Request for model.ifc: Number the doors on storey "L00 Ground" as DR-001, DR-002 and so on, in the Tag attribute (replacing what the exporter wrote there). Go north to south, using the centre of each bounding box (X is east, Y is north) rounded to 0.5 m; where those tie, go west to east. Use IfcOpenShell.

First a look at what the model holds.

```python
import ifcopenshell
import ifcopenshell.util.element
import ifcopenshell.util.placement

model = ifcopenshell.open("model.ifc")
print(model.schema)
storey = next(s for s in model.by_type("IfcBuildingStorey") if s.Name == "L00 Ground")
doors = [e for e in ifcopenshell.util.element.get_decomposition(storey) if e.is_a("IfcDoor")]
for e in sorted(doors, key=lambda e: e.id()):
    origin = ifcopenshell.util.placement.get_local_placement(e.ObjectPlacement)[:3, 3]
    print(e.id(), e.Tag, e.Name, origin.round(2) + 0.0, sep=" | ")
```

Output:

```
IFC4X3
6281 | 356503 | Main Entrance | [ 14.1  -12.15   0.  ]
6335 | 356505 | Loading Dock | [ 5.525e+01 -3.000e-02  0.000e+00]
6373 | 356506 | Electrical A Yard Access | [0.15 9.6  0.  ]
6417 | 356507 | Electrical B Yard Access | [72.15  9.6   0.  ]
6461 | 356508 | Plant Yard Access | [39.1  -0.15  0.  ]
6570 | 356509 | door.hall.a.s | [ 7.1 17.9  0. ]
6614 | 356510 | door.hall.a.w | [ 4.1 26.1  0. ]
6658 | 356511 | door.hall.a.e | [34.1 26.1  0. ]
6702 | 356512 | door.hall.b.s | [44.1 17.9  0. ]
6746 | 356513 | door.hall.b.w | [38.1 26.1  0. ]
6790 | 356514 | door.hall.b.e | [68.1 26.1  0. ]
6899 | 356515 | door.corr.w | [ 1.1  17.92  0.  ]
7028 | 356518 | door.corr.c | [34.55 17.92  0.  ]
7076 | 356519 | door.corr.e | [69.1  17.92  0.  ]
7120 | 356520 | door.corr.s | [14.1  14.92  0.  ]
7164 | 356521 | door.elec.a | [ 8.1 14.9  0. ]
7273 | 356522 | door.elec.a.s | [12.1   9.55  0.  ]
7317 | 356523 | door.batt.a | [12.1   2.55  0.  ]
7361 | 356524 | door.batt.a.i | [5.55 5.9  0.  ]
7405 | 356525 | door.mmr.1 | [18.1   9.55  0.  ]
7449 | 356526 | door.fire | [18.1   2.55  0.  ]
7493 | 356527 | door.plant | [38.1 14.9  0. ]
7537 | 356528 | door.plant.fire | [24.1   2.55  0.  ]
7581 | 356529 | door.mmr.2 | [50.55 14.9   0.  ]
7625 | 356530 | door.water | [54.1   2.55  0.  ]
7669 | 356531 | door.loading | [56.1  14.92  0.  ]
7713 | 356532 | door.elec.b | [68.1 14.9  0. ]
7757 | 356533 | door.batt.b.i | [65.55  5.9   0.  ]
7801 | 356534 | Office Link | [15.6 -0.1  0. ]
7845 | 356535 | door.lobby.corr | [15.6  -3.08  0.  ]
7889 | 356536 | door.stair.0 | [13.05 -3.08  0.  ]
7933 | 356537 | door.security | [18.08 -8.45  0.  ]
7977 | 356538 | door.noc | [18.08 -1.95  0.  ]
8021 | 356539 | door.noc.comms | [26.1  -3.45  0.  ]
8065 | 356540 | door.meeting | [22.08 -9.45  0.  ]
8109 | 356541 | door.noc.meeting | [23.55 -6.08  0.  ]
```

```python
import ifcopenshell
import ifcopenshell.geom
import ifcopenshell.util.element
import ifcopenshell.util.shape

model = ifcopenshell.open("model.ifc")
settings = ifcopenshell.geom.settings()
settings.set("use-world-coords", True)


def centre(element):
    shape = ifcopenshell.geom.create_shape(settings, element)
    return ifcopenshell.util.shape.get_bbox_centroid(shape.geometry)


storey = next(s for s in model.by_type("IfcBuildingStorey") if s.Name == "L00 Ground")
doors = [e for e in ifcopenshell.util.element.get_decomposition(storey) if e.is_a("IfcDoor")]

# Insertion points can sit at a corner or the storey origin, so sort by the geometry (in metres).
centres = {e: centre(e) for e in doors}
doors.sort(key=lambda e: (-round(centres[e][1] / 0.5), centres[e][0]))

for i, e in enumerate(doors, start=1):
    number = f"DR-0{i:02d}"
    e.Tag = number
    print(e.id(), number)

model.write("model_updated.ifc")
```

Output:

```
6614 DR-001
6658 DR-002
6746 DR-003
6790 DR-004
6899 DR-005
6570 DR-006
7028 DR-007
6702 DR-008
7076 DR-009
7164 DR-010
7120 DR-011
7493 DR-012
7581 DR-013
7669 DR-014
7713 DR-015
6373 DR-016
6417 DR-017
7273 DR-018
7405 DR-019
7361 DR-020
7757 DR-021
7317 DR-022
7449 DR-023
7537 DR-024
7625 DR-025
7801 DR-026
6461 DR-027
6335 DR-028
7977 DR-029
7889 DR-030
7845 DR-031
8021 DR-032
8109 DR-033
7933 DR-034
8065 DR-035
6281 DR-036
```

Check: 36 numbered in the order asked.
